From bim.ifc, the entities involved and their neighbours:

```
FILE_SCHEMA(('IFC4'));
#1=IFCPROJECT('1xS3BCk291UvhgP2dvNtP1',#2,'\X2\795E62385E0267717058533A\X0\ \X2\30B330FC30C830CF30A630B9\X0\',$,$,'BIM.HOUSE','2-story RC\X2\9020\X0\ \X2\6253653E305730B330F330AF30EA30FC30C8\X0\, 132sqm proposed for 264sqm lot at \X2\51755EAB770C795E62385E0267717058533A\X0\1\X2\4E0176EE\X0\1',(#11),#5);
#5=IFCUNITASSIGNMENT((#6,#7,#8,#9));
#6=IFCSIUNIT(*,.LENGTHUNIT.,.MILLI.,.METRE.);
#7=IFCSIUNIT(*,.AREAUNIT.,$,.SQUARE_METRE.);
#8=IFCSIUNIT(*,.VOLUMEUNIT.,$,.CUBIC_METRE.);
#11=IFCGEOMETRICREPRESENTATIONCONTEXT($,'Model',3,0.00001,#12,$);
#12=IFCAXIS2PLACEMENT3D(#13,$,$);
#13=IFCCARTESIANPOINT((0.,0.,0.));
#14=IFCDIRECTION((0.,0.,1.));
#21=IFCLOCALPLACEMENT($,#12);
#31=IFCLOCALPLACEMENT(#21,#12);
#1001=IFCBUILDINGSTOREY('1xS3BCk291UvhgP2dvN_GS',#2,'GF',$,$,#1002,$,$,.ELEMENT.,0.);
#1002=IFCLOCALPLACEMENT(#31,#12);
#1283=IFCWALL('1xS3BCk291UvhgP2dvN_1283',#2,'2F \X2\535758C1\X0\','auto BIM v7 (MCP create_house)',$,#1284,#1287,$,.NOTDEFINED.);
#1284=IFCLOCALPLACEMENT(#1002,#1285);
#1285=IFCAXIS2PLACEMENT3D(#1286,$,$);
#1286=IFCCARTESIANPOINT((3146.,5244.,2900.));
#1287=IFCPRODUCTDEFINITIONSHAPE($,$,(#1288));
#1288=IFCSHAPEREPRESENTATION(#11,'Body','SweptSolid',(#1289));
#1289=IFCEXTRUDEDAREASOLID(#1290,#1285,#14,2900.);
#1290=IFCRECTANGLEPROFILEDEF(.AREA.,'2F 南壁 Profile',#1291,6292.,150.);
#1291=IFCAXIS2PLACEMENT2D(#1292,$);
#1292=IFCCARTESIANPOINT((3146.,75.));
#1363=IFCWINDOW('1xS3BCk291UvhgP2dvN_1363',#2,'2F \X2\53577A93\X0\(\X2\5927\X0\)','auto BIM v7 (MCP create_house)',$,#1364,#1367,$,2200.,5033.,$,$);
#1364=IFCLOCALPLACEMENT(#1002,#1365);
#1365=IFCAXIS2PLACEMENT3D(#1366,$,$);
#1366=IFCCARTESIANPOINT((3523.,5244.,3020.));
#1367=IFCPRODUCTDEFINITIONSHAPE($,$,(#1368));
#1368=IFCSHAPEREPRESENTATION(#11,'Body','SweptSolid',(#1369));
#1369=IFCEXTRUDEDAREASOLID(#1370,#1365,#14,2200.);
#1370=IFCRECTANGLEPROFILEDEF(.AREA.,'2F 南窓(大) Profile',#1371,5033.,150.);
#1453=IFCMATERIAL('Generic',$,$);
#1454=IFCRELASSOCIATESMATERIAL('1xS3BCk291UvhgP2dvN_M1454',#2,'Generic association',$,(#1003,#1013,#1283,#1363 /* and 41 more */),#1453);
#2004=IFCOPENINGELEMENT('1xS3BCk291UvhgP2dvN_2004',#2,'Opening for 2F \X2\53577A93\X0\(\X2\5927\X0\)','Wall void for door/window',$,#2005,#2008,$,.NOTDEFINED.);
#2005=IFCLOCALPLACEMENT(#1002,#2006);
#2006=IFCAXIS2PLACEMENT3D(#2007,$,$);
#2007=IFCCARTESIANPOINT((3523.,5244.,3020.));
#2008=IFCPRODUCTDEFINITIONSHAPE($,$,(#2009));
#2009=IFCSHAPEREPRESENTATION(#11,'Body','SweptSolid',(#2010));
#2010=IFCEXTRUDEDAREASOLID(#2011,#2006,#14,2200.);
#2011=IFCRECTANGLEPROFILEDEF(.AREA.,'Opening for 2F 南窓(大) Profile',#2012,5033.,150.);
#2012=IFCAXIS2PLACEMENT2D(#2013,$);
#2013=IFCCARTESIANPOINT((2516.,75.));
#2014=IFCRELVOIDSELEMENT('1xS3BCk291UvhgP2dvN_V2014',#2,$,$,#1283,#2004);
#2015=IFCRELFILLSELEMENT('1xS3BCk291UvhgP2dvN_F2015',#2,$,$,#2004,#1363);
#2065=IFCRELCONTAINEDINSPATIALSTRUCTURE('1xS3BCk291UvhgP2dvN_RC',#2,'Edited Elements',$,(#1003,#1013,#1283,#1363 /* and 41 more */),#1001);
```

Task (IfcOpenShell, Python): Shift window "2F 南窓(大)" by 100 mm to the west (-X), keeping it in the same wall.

```python
import ifcopenshell
import ifcopenshell.api.geometry
import ifcopenshell.util.placement
import ifcopenshell.util.unit

model = ifcopenshell.open("bim.ifc")
unit_scale = ifcopenshell.util.unit.calculate_unit_scale(model)

window = model.by_guid("1xS3BCk291UvhgP2dvN_1363")
opening = window.FillsVoids[0].RelatingOpeningElement
wall = opening.VoidsElements[0].RelatingBuildingElement

wall_matrix = ifcopenshell.util.placement.get_local_placement(wall.ObjectPlacement)
shift = wall_matrix[:3, 0] * -0.1 / unit_scale
before = ifcopenshell.util.placement.get_local_placement(window.ObjectPlacement)[:3, 3].copy()

# The window is not placed relative to its opening, so move both.
for product in (opening, window):
    matrix = ifcopenshell.util.placement.get_local_placement(product.ObjectPlacement)
    matrix[:3, 3] += shift
    ifcopenshell.api.geometry.edit_object_placement(model, product=product, matrix=matrix, is_si=False)

after = ifcopenshell.util.placement.get_local_placement(window.ObjectPlacement)[:3, 3]
print("window moved by", (after - before).round(3) + 0.0)

model.write("bim_v2.ifc")
```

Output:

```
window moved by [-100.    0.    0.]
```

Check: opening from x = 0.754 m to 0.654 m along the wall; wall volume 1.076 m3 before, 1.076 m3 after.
